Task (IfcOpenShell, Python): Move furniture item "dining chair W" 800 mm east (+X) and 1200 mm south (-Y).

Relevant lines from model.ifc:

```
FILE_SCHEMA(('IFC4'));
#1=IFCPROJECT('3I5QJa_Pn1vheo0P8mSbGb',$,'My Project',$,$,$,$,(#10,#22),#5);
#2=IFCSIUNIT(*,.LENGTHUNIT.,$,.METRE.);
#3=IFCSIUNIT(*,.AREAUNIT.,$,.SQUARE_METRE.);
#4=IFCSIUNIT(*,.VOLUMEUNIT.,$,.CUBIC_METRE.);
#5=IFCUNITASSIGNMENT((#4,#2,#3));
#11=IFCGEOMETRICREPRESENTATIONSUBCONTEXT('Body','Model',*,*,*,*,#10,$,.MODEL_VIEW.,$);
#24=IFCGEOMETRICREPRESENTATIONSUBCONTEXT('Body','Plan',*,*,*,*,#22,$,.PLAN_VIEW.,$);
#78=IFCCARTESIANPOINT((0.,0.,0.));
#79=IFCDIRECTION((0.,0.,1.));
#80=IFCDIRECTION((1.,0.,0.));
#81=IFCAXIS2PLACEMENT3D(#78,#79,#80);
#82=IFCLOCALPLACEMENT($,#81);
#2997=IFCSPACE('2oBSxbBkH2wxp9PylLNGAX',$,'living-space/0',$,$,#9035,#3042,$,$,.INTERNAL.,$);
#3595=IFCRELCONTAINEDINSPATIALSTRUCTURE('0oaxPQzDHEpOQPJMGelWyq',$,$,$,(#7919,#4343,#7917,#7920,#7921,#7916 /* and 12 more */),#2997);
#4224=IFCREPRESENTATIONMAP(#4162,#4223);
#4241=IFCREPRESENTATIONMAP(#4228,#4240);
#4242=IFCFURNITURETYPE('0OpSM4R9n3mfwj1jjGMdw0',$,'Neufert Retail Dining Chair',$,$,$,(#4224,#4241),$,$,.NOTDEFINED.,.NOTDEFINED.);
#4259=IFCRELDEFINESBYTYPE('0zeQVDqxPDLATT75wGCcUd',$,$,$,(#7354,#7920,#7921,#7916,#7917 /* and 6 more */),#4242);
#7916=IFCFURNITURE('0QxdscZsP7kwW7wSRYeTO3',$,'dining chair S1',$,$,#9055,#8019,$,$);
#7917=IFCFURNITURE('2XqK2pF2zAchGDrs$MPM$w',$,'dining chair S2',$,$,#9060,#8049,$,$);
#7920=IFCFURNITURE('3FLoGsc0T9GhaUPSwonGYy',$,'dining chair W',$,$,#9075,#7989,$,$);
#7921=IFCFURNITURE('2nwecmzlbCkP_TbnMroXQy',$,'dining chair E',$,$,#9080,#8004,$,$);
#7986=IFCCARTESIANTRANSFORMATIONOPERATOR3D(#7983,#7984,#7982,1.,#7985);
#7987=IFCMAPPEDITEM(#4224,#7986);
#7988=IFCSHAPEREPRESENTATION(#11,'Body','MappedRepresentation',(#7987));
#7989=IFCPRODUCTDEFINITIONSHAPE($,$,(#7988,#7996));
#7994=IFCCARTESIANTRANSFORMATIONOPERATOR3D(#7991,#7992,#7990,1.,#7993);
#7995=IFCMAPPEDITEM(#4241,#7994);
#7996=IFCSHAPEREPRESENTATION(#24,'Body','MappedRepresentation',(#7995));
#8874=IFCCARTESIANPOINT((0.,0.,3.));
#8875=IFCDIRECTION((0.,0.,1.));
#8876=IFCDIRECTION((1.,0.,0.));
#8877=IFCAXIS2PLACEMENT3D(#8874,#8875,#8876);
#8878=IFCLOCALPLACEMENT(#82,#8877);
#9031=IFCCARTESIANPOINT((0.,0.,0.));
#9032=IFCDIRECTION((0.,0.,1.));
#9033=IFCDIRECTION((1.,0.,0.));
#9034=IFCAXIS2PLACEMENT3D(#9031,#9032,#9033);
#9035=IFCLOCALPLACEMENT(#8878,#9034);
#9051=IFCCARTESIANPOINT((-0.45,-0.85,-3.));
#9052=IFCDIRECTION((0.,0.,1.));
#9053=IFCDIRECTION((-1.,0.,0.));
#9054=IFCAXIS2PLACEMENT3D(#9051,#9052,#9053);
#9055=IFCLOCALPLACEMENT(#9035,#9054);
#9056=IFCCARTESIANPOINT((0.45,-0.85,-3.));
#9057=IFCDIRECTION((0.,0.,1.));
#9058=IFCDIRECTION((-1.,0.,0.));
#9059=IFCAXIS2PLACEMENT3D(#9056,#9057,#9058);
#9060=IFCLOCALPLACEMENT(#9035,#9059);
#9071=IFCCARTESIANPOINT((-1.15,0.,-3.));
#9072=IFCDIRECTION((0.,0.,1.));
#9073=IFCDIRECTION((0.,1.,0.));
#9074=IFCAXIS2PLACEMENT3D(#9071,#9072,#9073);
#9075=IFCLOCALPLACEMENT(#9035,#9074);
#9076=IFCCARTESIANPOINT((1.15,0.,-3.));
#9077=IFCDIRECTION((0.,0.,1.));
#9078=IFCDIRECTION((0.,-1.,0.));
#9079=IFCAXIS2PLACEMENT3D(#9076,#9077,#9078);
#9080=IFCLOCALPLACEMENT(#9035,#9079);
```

```python
import ifcopenshell
import ifcopenshell.api.geometry
import ifcopenshell.util.placement

model = ifcopenshell.open("model.ifc")

item = model.by_guid("3FLoGsc0T9GhaUPSwonGYy")
matrix = ifcopenshell.util.placement.get_local_placement(item.ObjectPlacement)
matrix[0, 3] += 0.8
matrix[1, 3] -= 1.2
ifcopenshell.api.geometry.edit_object_placement(model, product=item, matrix=matrix, is_si=False)

print(ifcopenshell.util.placement.get_local_placement(item.ObjectPlacement).round(3) + 0.0)

model.write("model_v2.ifc")
```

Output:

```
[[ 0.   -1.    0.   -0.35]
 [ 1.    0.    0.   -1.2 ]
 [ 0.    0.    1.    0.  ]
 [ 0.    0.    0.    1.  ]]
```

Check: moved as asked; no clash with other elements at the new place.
